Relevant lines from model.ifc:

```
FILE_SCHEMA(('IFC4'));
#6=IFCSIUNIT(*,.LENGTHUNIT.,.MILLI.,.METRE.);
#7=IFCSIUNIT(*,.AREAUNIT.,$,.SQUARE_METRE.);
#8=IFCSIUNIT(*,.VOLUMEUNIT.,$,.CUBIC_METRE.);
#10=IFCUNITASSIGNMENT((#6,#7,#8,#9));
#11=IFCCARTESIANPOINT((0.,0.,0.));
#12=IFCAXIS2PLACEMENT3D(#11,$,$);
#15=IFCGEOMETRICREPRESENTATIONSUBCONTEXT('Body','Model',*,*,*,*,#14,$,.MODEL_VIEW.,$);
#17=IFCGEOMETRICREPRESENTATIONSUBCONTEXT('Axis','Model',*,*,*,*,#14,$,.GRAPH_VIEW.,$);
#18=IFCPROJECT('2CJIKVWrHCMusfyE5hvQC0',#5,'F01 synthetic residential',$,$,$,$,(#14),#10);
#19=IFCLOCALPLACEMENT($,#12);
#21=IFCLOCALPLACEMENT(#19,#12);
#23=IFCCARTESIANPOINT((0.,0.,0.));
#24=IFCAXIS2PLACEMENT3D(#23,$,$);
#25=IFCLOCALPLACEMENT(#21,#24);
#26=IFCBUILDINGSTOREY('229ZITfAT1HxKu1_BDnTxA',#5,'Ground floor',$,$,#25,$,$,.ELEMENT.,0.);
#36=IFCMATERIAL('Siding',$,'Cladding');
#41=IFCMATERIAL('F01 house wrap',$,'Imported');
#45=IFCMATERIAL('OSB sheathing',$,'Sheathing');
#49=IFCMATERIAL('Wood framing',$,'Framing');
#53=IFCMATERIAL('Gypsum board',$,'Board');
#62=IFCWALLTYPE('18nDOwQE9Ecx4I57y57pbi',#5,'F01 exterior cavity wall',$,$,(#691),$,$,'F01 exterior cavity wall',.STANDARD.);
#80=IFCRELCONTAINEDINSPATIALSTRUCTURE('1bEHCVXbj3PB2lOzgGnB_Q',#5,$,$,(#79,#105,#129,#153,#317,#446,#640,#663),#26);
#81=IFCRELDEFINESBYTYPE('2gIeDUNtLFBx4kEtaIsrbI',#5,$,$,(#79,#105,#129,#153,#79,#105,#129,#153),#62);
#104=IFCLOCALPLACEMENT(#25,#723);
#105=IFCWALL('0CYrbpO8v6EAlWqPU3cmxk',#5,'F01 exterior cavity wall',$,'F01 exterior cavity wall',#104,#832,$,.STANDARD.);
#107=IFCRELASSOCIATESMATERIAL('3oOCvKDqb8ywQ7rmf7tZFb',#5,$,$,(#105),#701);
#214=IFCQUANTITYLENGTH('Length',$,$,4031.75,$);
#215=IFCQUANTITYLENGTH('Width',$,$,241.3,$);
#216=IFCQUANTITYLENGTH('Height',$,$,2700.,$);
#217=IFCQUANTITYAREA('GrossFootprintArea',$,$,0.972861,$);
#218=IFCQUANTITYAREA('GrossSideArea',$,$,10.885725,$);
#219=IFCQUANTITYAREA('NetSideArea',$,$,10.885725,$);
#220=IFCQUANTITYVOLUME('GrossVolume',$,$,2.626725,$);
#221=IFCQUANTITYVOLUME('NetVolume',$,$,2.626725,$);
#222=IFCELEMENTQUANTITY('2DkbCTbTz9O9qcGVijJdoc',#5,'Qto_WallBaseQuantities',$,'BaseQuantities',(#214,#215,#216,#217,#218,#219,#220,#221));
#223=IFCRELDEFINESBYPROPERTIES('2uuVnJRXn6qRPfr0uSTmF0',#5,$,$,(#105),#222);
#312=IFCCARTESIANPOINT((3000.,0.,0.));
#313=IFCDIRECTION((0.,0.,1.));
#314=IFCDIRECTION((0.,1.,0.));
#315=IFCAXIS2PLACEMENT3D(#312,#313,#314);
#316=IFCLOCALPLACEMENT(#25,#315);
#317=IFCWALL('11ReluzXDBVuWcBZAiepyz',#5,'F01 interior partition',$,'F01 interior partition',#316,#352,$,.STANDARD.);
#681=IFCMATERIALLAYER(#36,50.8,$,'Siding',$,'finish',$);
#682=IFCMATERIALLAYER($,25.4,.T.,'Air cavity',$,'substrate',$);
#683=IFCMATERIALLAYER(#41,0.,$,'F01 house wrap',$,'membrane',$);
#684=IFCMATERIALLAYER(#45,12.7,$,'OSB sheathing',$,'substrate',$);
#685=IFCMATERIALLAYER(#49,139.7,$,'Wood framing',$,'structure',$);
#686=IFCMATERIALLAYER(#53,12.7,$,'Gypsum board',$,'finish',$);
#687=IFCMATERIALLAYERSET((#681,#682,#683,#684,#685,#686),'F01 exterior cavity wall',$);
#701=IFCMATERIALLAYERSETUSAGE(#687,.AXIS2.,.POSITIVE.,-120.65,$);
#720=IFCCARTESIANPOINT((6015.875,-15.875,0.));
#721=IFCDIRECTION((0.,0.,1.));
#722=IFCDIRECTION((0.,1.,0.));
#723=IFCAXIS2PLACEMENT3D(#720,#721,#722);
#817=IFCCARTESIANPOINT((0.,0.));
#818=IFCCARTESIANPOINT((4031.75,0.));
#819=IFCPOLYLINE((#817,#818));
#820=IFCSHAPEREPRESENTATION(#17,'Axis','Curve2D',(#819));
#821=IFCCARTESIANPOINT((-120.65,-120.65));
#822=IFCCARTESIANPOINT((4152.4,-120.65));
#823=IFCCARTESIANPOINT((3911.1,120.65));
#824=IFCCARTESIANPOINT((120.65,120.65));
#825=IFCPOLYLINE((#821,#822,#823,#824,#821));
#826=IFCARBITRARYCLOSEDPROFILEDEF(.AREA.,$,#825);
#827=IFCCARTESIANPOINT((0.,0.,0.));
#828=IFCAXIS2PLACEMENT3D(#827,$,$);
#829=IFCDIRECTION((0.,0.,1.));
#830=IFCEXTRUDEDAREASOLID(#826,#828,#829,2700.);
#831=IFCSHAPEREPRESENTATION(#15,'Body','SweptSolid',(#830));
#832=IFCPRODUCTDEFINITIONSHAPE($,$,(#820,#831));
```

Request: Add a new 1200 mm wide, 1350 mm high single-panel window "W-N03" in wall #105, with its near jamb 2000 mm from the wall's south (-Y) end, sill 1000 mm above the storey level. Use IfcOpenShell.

```python
import numpy as np
import ifcopenshell
import ifcopenshell.api.feature
import ifcopenshell.api.geometry
import ifcopenshell.api.pset
import ifcopenshell.api.root
import ifcopenshell.api.spatial
import ifcopenshell.geom
import ifcopenshell.util.element
import ifcopenshell.util.placement
import ifcopenshell.util.representation
import ifcopenshell.util.shape
import ifcopenshell.util.unit

model = ifcopenshell.open("model.ifc")
unit_scale = ifcopenshell.util.unit.calculate_unit_scale(model)
area_scale = ifcopenshell.util.unit.calculate_unit_scale(model, "AREAUNIT")
volume_scale = ifcopenshell.util.unit.calculate_unit_scale(model, "VOLUMEUNIT")
settings = ifcopenshell.geom.settings()


def volume(element):
    """Net volume in cubic metres, openings subtracted."""
    shape = ifcopenshell.geom.create_shape(settings, element)
    return ifcopenshell.util.shape.get_volume(shape.geometry)


wall = model.by_guid("0CYrbpO8v6EAlWqPU3cmxk")
storey = ifcopenshell.util.element.get_container(wall, ifc_class="IfcBuildingStorey")
context = ifcopenshell.util.representation.get_context(model, "Model", "Body", "MODEL_VIEW")
before = volume(wall)

width, height, from_end, sill = 1.2, 1.35, 2, 1  # metres

# The wall runs along its own X axis, and the end named is its -X end.
wall_shape = ifcopenshell.geom.create_shape(settings, wall)
x, y, z = ifcopenshell.util.shape.get_vertices(wall_shape.geometry).T
start = x.min() + from_end
face, thickness = float(y.min()), float(y.max() - y.min())
wall_matrix = ifcopenshell.util.placement.get_local_placement(wall.ObjectPlacement)
level = ifcopenshell.util.placement.get_local_placement(storey.ObjectPlacement)[2, 3]


def in_wall(x, y):
    """Placement at x, y metres in the wall's axes, at sill height."""
    matrix = wall_matrix.copy()
    matrix[:, 3] = wall_matrix @ np.array([x / unit_scale, y / unit_scale, 0.0, 1.0])
    matrix[2, 3] = level + sill / unit_scale
    return matrix


# Opening: a box that overshoots both wall faces by 50 mm.
opening = ifcopenshell.api.root.create_entity(model, ifc_class="IfcOpeningElement", predefined_type="OPENING")
box = ifcopenshell.api.geometry.add_wall_representation(
    model, context=context, length=width, height=height, thickness=thickness + 0.1
)
ifcopenshell.api.geometry.assign_representation(model, product=opening, representation=box)
ifcopenshell.api.geometry.edit_object_placement(model, product=opening, matrix=in_wall(start, face - 0.05), is_si=False)
ifcopenshell.api.feature.add_feature(model, feature=opening, element=wall)

window = ifcopenshell.api.root.create_entity(model, ifc_class="IfcWindow", name="W-N03", predefined_type="WINDOW")
window.OverallWidth, window.OverallHeight = width / unit_scale, height / unit_scale
window.PartitioningType = "SINGLE_PANEL"
body = ifcopenshell.api.geometry.add_window_representation(
    model,
    context=context,
    overall_width=window.OverallWidth,
    overall_height=window.OverallHeight,
    partition_type="SINGLE_PANEL",
)
ifcopenshell.api.geometry.assign_representation(model, product=window, representation=body)
ifcopenshell.api.spatial.assign_container(model, products=[window], relating_structure=storey)
ifcopenshell.api.feature.add_filling(model, opening=opening, element=window)

# Centre the window in the wall's thickness.
ifcopenshell.api.geometry.edit_object_placement(model, product=window, matrix=in_wall(start, face), is_si=False)
window_shape = ifcopenshell.geom.create_shape(settings, window)
depth = ifcopenshell.util.shape.get_vertices(window_shape.geometry)[:, 1]
offset = face + thickness / 2 - (depth.min() + depth.max()) / 2
ifcopenshell.api.geometry.edit_object_placement(model, product=window, matrix=in_wall(start, offset), is_si=False)

after = volume(wall)

# Update the wall's stored quantities.
qto = model.by_id(ifcopenshell.util.element.get_pset(wall, "Qto_WallBaseQuantities", should_inherit=False)["id"])
ifcopenshell.api.pset.edit_qto(model, qto=qto, properties={
    "NetSideArea": after / thickness / area_scale,
    "NetVolume": after / volume_scale,
})

print(f"wall volume {before:.3f} -> {after:.3f} m3")

model.write("model-out.ifc")
```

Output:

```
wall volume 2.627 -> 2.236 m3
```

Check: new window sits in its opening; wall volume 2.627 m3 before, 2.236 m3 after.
